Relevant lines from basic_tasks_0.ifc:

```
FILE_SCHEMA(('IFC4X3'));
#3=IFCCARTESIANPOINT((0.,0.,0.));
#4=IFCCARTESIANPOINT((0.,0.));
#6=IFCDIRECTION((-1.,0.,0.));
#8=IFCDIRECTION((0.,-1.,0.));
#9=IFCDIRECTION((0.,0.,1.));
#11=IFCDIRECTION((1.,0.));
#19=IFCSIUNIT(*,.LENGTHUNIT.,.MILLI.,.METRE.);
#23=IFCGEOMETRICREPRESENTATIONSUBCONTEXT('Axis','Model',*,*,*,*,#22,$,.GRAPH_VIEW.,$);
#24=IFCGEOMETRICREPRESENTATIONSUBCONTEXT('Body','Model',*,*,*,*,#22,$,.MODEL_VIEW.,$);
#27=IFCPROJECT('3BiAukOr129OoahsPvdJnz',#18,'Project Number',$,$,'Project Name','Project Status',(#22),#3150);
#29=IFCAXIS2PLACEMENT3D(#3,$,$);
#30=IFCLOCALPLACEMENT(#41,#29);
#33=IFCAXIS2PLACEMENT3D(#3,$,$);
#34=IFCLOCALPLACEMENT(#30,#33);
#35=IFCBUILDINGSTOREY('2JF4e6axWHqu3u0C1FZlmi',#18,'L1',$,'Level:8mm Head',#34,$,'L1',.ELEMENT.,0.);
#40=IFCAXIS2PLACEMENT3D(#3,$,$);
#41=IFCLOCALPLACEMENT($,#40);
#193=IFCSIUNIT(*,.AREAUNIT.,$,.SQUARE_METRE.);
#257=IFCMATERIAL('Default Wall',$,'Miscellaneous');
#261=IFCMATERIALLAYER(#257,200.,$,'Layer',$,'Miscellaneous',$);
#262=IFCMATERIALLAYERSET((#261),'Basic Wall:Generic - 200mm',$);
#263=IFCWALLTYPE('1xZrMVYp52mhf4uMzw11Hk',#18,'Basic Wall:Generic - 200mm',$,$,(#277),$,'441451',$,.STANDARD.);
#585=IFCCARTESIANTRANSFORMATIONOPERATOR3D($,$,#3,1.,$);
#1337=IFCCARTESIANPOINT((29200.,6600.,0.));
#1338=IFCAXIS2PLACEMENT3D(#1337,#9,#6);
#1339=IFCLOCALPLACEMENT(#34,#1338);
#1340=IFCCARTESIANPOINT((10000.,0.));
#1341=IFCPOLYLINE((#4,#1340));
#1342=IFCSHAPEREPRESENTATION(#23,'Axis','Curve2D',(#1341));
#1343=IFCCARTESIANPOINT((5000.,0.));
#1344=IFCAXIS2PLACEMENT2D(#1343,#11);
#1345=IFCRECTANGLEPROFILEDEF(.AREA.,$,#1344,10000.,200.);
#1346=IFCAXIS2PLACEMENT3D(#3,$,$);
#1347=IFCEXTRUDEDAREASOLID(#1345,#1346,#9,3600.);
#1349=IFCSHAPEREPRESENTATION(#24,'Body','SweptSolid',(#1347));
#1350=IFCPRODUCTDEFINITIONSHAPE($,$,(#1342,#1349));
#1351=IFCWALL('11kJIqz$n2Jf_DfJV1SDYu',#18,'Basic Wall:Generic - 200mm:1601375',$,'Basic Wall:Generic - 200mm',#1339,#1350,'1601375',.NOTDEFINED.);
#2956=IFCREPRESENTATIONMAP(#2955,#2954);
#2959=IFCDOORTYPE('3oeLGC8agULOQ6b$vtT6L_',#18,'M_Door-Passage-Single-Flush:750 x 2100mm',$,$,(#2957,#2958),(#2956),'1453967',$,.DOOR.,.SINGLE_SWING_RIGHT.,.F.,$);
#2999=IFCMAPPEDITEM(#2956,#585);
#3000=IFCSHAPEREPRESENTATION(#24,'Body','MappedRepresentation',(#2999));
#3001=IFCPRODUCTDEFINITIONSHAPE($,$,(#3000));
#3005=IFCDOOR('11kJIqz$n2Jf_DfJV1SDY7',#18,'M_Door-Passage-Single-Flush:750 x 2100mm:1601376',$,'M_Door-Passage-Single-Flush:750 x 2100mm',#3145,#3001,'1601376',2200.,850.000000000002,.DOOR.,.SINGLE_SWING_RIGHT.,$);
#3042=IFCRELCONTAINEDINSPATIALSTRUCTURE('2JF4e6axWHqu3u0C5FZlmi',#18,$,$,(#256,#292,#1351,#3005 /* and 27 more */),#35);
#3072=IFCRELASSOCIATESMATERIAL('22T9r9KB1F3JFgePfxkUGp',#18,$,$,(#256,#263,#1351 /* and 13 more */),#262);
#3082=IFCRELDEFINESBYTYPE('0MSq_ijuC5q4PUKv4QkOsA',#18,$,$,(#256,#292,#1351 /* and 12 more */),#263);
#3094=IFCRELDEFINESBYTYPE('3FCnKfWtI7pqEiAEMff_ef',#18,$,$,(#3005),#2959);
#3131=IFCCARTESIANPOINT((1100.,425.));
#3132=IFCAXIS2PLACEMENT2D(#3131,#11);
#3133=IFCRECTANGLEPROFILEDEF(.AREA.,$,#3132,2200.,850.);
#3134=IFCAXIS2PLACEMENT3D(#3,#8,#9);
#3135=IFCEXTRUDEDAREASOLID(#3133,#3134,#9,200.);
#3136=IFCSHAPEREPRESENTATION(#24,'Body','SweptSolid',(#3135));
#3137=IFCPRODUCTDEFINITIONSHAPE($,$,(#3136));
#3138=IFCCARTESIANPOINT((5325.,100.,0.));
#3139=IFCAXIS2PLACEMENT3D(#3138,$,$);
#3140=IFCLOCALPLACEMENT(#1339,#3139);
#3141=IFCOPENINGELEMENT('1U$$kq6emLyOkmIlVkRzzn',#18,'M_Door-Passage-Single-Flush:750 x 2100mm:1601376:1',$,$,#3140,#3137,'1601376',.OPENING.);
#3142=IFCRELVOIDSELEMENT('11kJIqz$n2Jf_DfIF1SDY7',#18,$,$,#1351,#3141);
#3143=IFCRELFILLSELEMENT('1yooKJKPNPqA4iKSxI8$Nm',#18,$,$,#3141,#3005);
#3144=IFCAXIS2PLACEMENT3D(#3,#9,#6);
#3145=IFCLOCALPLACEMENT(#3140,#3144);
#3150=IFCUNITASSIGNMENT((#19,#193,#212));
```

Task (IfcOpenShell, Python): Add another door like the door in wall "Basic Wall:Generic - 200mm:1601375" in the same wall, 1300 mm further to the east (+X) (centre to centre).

```python
import ifcopenshell
import ifcopenshell.api.feature
import ifcopenshell.api.geometry
import ifcopenshell.api.root
import ifcopenshell.geom
import ifcopenshell.util.element
import ifcopenshell.util.placement
import ifcopenshell.util.shape

model = ifcopenshell.open("basic_tasks_0.ifc")
settings = ifcopenshell.geom.settings()


def volume(element):
    """Net volume in cubic metres, openings subtracted."""
    shape = ifcopenshell.geom.create_shape(settings, element)
    return ifcopenshell.util.shape.get_volume(shape.geometry)


def reuse_history(source, copy):
    """copy_class also copies each property set's owner history, people and application; keep the originals."""
    for rel in copy.IsDefinedBy:
        if rel.is_a("IfcRelDefinesByProperties") and (history := rel.RelatingPropertyDefinition.OwnerHistory):
            rel.RelatingPropertyDefinition.OwnerHistory = source.OwnerHistory
            ifcopenshell.util.element.remove_deep2(model, history)


door = model.by_id(3005)
opening = door.FillsVoids[0].RelatingOpeningElement
wall = opening.VoidsElements[0].RelatingBuildingElement
before = volume(wall)
shift = ifcopenshell.util.placement.get_local_placement(wall.ObjectPlacement)[:3, 0] * -1300.0

# copy_class copies the void relationship, type, container and properties, but no geometry.
new_opening = ifcopenshell.api.root.copy_class(model, product=opening)
new_opening.Representation = ifcopenshell.util.element.copy_deep(
    model, opening.Representation, exclude=["IfcGeometricRepresentationContext", "IfcRepresentationMap"]
)
new_opening.Name = "M_Door-Passage-Single-Flush:750 x 2100mm"
new_opening.Tag = None
new_door = ifcopenshell.api.root.copy_class(model, product=door)
new_door.Representation = ifcopenshell.util.element.copy_deep(
    model, door.Representation, exclude=["IfcGeometricRepresentationContext", "IfcRepresentationMap"]
)
new_door.Name = "M_Door-Passage-Single-Flush:750 x 2100mm"
new_door.Tag = None
reuse_history(door, new_door)
ifcopenshell.api.feature.add_filling(model, opening=new_opening, element=new_door)

for old, new in ((opening, new_opening), (door, new_door)):
    matrix = ifcopenshell.util.placement.get_local_placement(old.ObjectPlacement)
    matrix[:3, 3] += shift
    ifcopenshell.api.geometry.edit_object_placement(model, product=new, matrix=matrix, is_si=False)

after = volume(wall)

print(f"wall volume {before:.3f} -> {after:.3f} m3")

model.write("basic_tasks_0_v2.ifc")
```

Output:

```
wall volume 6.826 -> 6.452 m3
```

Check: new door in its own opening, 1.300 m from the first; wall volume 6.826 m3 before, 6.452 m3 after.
